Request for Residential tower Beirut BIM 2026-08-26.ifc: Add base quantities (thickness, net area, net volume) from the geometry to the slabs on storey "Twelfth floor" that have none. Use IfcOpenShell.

First a look at what the model holds.

```python
import ifcopenshell
import ifcopenshell.util.element
import ifcopenshell.util.unit

model = ifcopenshell.open("Residential tower Beirut BIM 2026-08-26.ifc")
print(model.schema)
for unit_type in ("LENGTHUNIT", "AREAUNIT", "VOLUMEUNIT"):
    print(unit_type, ifcopenshell.util.unit.calculate_unit_scale(model, unit_type))
storey = next(s for s in model.by_type("IfcBuildingStorey") if s.Name == "Twelfth floor")
slabs = [e for e in ifcopenshell.util.element.get_decomposition(storey) if e.is_a("IfcSlab")]
for e in sorted(slabs, key=lambda e: e.id()):
    print(e.id(), e.is_a(), e.Name, list(ifcopenshell.util.element.get_psets(e, qtos_only=True)), sep=" | ")
```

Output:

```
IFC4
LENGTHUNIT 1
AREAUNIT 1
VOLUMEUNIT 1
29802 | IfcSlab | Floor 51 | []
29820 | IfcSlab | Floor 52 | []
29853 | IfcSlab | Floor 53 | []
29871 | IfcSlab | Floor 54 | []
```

```python
import ifcopenshell
import ifcopenshell.api.pset
import ifcopenshell.geom
import ifcopenshell.util.element
import ifcopenshell.util.shape
import ifcopenshell.util.unit

model = ifcopenshell.open("Residential tower Beirut BIM 2026-08-26.ifc")
unit_scale = ifcopenshell.util.unit.calculate_unit_scale(model)
area_scale = ifcopenshell.util.unit.calculate_unit_scale(model, "AREAUNIT")
volume_scale = ifcopenshell.util.unit.calculate_unit_scale(model, "VOLUMEUNIT")
settings = ifcopenshell.geom.settings()

storey = next(s for s in model.by_type("IfcBuildingStorey") if s.Name == "Twelfth floor")
slabs = [e for e in ifcopenshell.util.element.get_decomposition(storey) if e.is_a("IfcSlab")]

for e in sorted(slabs, key=lambda e: e.id()):
    if ifcopenshell.util.element.get_psets(e, qtos_only=True, should_inherit=False):
        continue
    # Geometry comes back in metres, in the element's own axes.
    shape = ifcopenshell.geom.create_shape(settings, e)
    values = {
        "Width": ifcopenshell.util.shape.get_z(shape.geometry) / unit_scale,
        "NetArea": ifcopenshell.util.shape.get_footprint_area(shape.geometry) / area_scale,
        "NetVolume": ifcopenshell.util.shape.get_volume(shape.geometry) / volume_scale,
    }
    qto = ifcopenshell.api.pset.add_qto(model, product=e, name="Qto_SlabBaseQuantities")
    ifcopenshell.api.pset.edit_qto(model, qto=qto, properties=values)
    print(e.id(), {k: round(v, 3) for k, v in values.items()})

model.write("Residential tower Beirut BIM 2026-08-26_updated.ifc")
```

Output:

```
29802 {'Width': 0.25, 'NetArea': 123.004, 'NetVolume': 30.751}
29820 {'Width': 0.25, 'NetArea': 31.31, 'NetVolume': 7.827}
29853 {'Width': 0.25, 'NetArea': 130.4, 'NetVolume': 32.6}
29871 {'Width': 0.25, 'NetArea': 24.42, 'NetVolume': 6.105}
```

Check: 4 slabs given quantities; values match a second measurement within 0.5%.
